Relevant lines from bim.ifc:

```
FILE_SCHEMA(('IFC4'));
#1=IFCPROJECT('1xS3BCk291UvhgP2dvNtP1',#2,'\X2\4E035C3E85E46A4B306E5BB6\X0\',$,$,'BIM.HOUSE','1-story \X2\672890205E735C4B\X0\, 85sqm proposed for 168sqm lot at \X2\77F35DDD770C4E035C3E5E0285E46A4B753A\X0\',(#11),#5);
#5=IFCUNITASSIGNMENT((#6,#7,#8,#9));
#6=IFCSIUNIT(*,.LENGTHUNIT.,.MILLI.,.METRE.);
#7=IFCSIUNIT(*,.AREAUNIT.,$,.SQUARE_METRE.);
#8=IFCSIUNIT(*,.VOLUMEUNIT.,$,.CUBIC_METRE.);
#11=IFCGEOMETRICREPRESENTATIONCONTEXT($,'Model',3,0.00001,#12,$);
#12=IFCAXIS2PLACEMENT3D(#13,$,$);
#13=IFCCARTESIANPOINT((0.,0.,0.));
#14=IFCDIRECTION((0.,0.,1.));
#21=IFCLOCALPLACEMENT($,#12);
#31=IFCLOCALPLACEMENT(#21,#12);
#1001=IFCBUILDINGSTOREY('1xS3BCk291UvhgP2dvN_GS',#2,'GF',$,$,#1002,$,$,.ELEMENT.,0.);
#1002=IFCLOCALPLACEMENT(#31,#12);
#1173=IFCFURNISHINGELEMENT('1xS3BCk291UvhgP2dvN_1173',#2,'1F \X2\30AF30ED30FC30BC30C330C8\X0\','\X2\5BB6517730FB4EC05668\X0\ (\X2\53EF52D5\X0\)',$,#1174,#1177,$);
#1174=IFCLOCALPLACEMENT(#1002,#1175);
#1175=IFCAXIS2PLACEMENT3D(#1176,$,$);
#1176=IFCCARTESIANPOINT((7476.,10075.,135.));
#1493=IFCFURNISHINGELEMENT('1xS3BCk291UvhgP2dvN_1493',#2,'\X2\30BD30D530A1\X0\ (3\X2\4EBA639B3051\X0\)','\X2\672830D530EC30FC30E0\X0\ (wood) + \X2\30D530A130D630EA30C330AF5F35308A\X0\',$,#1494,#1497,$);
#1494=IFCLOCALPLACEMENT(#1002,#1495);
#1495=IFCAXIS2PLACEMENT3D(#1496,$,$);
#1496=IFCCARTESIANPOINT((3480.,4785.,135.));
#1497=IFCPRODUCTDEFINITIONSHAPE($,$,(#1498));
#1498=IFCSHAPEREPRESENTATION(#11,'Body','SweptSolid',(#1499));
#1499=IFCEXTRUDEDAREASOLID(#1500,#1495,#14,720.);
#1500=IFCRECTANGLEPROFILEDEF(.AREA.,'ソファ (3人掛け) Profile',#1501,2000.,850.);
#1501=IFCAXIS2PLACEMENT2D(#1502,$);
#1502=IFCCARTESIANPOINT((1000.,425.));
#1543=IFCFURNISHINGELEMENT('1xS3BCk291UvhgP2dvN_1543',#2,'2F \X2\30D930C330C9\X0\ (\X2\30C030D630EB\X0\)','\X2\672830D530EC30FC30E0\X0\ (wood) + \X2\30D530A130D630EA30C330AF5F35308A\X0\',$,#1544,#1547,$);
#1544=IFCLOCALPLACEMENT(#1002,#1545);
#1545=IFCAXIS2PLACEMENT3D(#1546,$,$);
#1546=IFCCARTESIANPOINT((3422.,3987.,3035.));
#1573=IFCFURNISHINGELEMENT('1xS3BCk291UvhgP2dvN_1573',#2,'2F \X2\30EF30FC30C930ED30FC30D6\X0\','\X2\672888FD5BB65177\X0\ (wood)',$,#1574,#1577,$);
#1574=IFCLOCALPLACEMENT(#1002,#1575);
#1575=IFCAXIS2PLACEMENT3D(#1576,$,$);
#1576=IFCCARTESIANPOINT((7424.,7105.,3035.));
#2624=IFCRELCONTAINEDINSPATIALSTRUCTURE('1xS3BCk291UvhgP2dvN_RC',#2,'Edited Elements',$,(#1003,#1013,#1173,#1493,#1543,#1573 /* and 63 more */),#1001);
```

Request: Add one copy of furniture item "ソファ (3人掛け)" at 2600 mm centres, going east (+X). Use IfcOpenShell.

```python
import numpy as np
import ifcopenshell
import ifcopenshell.api.geometry
import ifcopenshell.api.root
import ifcopenshell.util.element
import ifcopenshell.util.placement
import ifcopenshell.util.unit

model = ifcopenshell.open("bim.ifc")
unit_scale = ifcopenshell.util.unit.calculate_unit_scale(model)


def reuse_history(source, copy):
    """copy_class also copies each property set's owner history, people and application; keep the originals."""
    for rel in copy.IsDefinedBy:
        if rel.is_a("IfcRelDefinesByProperties") and (history := rel.RelatingPropertyDefinition.OwnerHistory):
            rel.RelatingPropertyDefinition.OwnerHistory = source.OwnerHistory
            ifcopenshell.util.element.remove_deep2(model, history)


source = model.by_guid("1xS3BCk291UvhgP2dvN_1493")
base = ifcopenshell.util.placement.get_local_placement(source.ObjectPlacement)
step = np.array([1.0, 0.0, 0.0]) * 2.6 / unit_scale

for i in range(1, 2):
    copy = ifcopenshell.api.root.copy_class(model, product=source)
    copy.Representation = ifcopenshell.util.element.copy_deep(
        model, source.Representation, exclude=["IfcGeometricRepresentationContext", "IfcRepresentationMap"]
    )
    reuse_history(source, copy)
    matrix = base.copy()
    matrix[:3, 3] += i * step
    print("added at", matrix[:3, 3].round(3) + 0.0)
    ifcopenshell.api.geometry.edit_object_placement(model, product=copy, matrix=matrix, is_si=False)

model.write("bim-out.ifc")
```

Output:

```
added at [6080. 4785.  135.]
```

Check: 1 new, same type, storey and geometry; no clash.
